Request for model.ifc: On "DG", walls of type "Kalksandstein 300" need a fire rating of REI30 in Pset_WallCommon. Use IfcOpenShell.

First a look at what the model holds.

```python
import ifcopenshell
import ifcopenshell.util.element

model = ifcopenshell.open("model.ifc")
print(model.schema)
storey = next(s for s in model.by_type("IfcBuildingStorey") if s.Name == "DG")
walls = [e for e in ifcopenshell.util.element.get_decomposition(storey) if e.is_a("IfcWall")]
seen = {}
for e in walls:
    element_type = ifcopenshell.util.element.get_type(e)
    key = (element_type.Name if element_type != e and element_type else None, ifcopenshell.util.element.get_pset(e, "Pset_WallCommon", "FireRating"))
    seen[key] = seen.get(key, 0) + 1
for (name, value), count in sorted(seen.items(), key=str):
    print(count, "x", name, "|", value)
```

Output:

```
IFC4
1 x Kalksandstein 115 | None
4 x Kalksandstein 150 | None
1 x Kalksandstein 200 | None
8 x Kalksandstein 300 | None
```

```python
import ifcopenshell
import ifcopenshell.api.pset
import ifcopenshell.util.element

model = ifcopenshell.open("model.ifc")

storey = next(s for s in model.by_type("IfcBuildingStorey") if s.Name == "DG")
walls = [e for e in ifcopenshell.util.element.get_decomposition(storey) if e.is_a("IfcWall")]

count = 0
for e in walls:
    element_type = ifcopenshell.util.element.get_type(e)
    if element_type in (None, e) or element_type.Name != "Kalksandstein 300":
        continue
    # add_pset returns the element's existing set when there is one.
    pset = ifcopenshell.api.pset.add_pset(model, product=e, name="Pset_WallCommon")
    ifcopenshell.api.pset.edit_pset(model, pset=pset, properties={"FireRating": "REI30"})
    count += 1

print(count, "walls updated")

model.write("model_edited.ifc")
```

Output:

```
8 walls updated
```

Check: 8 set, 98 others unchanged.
